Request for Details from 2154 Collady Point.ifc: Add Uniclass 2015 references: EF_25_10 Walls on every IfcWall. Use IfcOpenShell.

First a look at what the model holds.

```python
import ifcopenshell

model = ifcopenshell.open("Details from 2154 Collady Point.ifc")
print(model.schema)
print("classifications:", [c.Name for c in model.by_type("IfcClassification")])
for ifc_class in ("IfcDoor", "IfcRoof", "IfcStair", "IfcWall", "IfcWindow"):
    print(ifc_class, len(model.by_type(ifc_class)))
```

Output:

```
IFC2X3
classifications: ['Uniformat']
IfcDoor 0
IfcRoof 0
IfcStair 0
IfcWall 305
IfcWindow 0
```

```python
import ifcopenshell
import ifcopenshell.api.classification

model = ifcopenshell.open("Details from 2154 Collady Point.ifc")

# IFC2X3 requires Source and Edition and has no link from the project to the system.
system = model.create_entity("IfcClassification", Source="NBS", Edition="2015", Name="Uniclass 2015")

codes = {
    "IfcWall": ("EF_25_10", "Walls"),
}
for ifc_class, (code, name) in codes.items():
    products = model.by_type(ifc_class)
    ifcopenshell.api.classification.add_reference(
        model, products=products, classification=system, identification=code, name=name
    )
    print(code, len(products))

model.write("Details from 2154 Collady Point_v2.ifc")
```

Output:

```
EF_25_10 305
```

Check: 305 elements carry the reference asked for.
